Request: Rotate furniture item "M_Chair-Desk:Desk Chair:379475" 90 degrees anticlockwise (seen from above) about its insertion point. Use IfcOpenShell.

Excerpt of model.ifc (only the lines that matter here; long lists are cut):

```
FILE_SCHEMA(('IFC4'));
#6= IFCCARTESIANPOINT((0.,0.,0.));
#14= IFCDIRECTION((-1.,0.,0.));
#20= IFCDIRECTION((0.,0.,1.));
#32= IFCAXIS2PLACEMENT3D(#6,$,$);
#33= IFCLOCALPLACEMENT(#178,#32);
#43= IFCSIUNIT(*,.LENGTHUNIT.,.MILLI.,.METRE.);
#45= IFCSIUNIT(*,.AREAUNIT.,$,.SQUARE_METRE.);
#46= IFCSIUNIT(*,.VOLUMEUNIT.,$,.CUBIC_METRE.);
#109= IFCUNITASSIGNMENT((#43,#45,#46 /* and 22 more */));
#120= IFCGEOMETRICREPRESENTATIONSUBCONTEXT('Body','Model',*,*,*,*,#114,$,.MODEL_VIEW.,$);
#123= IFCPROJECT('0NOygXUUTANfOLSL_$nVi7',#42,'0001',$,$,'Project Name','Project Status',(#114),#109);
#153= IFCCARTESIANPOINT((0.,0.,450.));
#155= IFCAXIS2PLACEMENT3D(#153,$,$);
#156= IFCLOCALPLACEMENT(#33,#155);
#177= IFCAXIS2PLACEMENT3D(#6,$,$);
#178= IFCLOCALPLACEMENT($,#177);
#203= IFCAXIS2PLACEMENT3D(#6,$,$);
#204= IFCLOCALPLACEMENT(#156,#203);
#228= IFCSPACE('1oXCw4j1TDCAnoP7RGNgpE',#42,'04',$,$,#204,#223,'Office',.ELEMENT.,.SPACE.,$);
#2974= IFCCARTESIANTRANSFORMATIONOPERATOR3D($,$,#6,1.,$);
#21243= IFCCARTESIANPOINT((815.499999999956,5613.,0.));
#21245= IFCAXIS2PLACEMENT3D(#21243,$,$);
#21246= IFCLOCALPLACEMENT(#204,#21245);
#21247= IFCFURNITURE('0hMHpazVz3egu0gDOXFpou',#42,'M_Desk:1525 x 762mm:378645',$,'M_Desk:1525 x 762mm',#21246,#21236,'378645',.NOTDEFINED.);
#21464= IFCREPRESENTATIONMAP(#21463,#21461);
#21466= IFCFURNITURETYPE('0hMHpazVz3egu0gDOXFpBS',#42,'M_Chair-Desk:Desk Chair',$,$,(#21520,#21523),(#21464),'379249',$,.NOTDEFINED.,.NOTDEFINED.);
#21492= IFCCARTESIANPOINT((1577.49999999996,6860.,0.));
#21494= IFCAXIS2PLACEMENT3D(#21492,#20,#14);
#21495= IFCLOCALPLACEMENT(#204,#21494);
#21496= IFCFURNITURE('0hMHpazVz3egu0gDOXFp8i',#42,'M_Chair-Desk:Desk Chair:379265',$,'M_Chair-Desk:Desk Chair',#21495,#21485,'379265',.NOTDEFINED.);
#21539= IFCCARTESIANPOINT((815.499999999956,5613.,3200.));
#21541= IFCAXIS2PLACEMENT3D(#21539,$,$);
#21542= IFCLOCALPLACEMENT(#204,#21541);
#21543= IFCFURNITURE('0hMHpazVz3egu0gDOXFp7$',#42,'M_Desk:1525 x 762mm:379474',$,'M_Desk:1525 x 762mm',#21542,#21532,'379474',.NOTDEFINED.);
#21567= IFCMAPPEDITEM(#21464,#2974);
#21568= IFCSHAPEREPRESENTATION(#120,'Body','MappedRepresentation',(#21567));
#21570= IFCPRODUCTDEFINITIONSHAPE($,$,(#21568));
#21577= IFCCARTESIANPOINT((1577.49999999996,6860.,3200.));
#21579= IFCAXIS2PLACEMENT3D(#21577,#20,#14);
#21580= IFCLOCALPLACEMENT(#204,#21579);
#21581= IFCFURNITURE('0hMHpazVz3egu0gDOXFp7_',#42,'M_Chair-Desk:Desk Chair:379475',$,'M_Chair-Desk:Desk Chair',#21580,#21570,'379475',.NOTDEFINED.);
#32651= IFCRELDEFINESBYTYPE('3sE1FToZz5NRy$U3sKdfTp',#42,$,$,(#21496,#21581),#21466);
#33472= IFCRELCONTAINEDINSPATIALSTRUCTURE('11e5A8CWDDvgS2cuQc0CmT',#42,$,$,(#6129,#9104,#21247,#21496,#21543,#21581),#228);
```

```python
import ifcopenshell
import ifcopenshell.api.geometry
import ifcopenshell.util.placement

model = ifcopenshell.open("model.ifc")

item = model.by_id(21581)
matrix = ifcopenshell.util.placement.get_local_placement(item.ObjectPlacement)
matrix = matrix @ ifcopenshell.util.placement.rotation(90, "Z")
ifcopenshell.api.geometry.edit_object_placement(model, product=item, matrix=matrix, is_si=False)

print(ifcopenshell.util.placement.get_local_placement(item.ObjectPlacement).round(3) + 0.0)

model.write("model_rev.ifc")
```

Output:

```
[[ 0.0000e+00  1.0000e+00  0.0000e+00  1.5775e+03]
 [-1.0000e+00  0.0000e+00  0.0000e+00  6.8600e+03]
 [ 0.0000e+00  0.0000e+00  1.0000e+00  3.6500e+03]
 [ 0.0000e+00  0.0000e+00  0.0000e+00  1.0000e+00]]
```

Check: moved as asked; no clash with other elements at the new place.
